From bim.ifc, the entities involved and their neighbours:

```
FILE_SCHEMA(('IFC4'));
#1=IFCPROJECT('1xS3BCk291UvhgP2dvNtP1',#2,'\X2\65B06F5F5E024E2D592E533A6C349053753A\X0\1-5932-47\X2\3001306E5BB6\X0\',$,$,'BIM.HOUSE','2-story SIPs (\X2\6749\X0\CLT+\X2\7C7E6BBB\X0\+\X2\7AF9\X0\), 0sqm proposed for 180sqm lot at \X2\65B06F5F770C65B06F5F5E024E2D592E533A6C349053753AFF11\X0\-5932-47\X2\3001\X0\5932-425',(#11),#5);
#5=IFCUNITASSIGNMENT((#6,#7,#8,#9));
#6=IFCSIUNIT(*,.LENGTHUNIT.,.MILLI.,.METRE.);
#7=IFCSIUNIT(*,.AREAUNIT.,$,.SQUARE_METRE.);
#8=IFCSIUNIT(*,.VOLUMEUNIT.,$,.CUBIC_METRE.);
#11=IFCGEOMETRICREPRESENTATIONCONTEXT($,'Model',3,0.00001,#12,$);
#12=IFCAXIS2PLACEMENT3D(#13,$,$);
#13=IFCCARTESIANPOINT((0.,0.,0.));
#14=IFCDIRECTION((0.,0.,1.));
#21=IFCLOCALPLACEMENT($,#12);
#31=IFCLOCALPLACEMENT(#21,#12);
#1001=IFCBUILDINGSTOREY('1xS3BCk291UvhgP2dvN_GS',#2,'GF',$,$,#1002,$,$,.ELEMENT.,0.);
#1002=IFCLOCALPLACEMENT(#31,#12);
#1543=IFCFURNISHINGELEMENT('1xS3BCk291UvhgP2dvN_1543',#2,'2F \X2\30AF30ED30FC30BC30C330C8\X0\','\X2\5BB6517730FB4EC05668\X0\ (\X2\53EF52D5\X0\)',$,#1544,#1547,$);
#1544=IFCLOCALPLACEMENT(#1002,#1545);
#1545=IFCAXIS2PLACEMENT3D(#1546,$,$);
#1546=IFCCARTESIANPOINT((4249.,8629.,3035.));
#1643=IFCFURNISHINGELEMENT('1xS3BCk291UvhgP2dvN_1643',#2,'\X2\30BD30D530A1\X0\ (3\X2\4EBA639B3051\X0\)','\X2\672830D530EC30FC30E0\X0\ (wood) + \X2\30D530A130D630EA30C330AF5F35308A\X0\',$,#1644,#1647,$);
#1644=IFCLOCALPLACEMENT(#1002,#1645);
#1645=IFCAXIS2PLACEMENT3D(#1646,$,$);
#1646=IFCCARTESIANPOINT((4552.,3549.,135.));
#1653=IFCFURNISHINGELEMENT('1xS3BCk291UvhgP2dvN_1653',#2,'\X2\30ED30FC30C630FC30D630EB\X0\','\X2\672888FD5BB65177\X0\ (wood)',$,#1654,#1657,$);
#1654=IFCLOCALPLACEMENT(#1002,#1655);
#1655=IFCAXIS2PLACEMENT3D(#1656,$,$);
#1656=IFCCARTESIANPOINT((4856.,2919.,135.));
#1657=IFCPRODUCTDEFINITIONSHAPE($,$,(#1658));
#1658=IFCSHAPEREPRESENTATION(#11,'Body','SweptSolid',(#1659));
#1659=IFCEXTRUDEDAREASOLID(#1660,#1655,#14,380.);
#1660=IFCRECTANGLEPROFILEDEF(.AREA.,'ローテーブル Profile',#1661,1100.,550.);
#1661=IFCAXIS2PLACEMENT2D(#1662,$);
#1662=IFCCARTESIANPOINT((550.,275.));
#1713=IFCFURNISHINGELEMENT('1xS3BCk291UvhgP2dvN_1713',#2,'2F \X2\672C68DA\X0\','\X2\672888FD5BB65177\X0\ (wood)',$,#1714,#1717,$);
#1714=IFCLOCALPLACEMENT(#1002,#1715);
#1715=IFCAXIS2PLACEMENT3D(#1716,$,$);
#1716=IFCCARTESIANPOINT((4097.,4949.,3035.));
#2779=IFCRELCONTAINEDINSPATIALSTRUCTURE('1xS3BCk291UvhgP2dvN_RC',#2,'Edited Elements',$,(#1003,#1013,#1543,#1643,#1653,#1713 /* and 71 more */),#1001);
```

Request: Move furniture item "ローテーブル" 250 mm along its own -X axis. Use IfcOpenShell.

```python
import ifcopenshell
import ifcopenshell.api.geometry
import ifcopenshell.util.placement

model = ifcopenshell.open("bim.ifc")

item = model.by_guid("1xS3BCk291UvhgP2dvN_1653")
matrix = ifcopenshell.util.placement.get_local_placement(item.ObjectPlacement)
matrix[:3, 3] -= matrix[:3, 0] * 250.0
ifcopenshell.api.geometry.edit_object_placement(model, product=item, matrix=matrix, is_si=False)

print(ifcopenshell.util.placement.get_local_placement(item.ObjectPlacement).round(3) + 0.0)

model.write("bim-out.ifc")
```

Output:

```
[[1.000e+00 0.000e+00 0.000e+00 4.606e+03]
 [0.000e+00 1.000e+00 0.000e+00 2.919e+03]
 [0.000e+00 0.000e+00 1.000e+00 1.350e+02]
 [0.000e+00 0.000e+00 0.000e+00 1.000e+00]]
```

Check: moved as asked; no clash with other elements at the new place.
